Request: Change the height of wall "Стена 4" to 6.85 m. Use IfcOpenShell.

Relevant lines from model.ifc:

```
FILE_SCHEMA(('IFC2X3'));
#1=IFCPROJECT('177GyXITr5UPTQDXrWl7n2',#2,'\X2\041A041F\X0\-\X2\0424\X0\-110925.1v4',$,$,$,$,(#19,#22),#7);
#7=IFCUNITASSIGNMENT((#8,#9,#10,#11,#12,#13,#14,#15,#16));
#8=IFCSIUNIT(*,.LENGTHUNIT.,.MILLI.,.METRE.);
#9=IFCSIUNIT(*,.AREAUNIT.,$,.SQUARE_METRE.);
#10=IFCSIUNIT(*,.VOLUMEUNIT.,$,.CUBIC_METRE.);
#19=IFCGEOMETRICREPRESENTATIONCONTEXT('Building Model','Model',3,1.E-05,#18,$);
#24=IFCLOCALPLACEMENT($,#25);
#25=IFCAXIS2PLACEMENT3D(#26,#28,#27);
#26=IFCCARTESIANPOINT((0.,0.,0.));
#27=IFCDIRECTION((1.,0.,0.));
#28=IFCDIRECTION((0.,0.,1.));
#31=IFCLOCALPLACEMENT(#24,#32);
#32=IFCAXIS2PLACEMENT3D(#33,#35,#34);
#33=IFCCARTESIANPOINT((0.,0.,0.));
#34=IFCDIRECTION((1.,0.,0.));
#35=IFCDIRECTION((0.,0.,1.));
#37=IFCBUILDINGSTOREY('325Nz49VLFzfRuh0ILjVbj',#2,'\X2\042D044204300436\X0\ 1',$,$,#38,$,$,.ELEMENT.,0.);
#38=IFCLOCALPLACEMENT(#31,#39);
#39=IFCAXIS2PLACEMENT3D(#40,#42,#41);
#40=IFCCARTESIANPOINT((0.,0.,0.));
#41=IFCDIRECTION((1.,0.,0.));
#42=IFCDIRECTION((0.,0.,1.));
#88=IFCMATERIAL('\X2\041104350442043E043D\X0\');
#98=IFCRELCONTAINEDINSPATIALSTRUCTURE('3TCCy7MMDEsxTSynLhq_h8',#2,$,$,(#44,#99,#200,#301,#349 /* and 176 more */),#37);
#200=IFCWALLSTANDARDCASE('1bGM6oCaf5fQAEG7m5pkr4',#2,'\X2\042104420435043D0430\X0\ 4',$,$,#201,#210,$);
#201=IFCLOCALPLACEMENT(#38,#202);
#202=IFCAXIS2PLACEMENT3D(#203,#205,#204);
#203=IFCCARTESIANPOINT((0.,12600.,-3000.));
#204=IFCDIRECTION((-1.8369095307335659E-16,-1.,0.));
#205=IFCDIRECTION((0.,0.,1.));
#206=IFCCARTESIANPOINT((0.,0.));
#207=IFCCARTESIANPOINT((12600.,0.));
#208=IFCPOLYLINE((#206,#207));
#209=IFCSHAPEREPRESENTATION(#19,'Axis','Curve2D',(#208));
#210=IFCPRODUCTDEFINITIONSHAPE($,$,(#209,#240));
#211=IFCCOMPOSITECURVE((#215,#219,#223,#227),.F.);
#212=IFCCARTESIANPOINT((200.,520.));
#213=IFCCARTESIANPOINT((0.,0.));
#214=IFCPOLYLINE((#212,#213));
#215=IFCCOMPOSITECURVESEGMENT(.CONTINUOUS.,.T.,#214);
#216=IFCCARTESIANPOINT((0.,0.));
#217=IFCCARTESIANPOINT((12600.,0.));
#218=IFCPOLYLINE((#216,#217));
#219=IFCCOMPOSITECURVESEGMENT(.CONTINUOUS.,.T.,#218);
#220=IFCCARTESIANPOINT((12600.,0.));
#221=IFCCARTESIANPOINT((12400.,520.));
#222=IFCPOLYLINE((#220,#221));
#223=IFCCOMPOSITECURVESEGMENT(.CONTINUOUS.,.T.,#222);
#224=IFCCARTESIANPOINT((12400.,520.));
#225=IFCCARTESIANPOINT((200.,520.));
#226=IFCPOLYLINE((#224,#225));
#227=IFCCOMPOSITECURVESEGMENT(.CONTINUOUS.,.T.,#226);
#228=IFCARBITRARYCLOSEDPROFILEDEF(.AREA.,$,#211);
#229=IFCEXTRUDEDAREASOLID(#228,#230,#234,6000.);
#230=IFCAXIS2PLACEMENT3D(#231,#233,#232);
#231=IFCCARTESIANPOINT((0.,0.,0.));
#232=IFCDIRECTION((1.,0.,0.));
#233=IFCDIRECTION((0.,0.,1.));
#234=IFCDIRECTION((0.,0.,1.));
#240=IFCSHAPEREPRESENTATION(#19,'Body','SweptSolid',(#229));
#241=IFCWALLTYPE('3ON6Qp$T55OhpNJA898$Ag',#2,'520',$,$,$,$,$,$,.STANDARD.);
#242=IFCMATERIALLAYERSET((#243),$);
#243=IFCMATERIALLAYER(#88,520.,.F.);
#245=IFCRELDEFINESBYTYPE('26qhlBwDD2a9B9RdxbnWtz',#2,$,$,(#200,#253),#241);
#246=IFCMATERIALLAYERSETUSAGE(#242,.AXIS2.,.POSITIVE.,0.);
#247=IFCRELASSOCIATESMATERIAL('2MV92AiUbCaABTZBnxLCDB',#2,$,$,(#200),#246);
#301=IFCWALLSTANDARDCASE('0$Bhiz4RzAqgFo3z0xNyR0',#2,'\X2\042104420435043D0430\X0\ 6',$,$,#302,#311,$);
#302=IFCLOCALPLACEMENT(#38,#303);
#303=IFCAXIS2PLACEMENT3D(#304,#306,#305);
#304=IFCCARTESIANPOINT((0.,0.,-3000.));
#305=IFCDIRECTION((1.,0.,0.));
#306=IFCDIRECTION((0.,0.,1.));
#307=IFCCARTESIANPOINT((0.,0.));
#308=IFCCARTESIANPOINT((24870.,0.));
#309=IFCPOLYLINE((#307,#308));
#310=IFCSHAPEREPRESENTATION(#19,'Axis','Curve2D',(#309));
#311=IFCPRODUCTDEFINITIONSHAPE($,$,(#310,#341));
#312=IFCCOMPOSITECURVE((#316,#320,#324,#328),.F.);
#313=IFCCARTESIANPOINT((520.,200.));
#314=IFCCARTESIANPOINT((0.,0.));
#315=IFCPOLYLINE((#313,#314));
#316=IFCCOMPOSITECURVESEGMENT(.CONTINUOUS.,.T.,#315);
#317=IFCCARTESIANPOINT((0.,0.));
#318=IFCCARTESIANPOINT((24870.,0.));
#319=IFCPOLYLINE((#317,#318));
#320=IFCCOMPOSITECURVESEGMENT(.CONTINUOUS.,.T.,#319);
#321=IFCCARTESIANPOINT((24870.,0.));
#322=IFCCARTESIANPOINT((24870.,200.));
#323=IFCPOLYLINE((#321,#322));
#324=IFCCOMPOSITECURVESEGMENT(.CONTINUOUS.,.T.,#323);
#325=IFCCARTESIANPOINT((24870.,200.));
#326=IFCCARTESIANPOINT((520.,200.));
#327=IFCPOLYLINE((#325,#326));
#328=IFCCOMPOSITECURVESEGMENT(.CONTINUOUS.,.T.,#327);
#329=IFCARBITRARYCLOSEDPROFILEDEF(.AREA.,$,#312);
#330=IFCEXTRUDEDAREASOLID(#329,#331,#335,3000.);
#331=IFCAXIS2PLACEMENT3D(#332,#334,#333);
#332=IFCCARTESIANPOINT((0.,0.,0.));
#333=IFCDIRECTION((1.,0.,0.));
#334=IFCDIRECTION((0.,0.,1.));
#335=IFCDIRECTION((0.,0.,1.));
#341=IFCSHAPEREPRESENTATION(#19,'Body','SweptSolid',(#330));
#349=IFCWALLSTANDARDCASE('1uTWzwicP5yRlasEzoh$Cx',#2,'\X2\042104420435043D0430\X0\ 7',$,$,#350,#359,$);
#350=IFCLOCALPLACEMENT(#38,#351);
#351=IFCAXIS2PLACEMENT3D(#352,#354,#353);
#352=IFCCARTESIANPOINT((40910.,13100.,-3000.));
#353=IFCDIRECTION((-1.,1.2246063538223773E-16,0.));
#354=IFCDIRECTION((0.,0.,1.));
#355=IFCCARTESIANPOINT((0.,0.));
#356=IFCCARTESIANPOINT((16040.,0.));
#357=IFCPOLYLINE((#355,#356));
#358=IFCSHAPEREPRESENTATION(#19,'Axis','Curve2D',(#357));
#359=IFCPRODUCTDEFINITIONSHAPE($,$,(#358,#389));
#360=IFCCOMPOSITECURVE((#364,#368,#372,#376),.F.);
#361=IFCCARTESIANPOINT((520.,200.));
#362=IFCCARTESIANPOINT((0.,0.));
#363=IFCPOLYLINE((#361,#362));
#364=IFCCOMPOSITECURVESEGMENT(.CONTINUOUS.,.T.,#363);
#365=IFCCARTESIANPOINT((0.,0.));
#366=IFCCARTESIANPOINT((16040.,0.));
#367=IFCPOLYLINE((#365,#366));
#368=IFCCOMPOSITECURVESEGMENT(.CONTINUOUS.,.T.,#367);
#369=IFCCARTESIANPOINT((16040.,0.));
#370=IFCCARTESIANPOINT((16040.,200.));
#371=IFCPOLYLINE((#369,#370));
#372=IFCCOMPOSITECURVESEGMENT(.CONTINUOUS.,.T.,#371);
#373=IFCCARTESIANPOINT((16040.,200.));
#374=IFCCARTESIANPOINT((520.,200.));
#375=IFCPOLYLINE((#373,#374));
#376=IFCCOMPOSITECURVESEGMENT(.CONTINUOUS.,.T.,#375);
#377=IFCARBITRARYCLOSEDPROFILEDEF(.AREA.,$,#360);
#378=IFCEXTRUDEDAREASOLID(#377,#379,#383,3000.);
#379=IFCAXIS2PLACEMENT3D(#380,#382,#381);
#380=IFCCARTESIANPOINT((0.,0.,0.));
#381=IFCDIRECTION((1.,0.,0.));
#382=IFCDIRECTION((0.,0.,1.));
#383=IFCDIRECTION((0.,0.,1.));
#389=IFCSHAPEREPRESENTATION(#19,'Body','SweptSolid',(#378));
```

```python
import ifcopenshell
import ifcopenshell.geom
import ifcopenshell.util.shape

model = ifcopenshell.open("model.ifc")
settings = ifcopenshell.geom.settings()


def volume(element):
    """Net volume in cubic metres, openings subtracted."""
    shape = ifcopenshell.geom.create_shape(settings, element)
    return ifcopenshell.util.shape.get_volume(shape.geometry)


wall = model.by_guid("1bGM6oCaf5fQAEG7m5pkr4")
before = volume(wall)

body = next(r for r in wall.Representation.Representations if r.RepresentationIdentifier == "Body")
solid = body.Items[0]
old_height = solid.Depth
solid.Depth = 6850.0
after = volume(wall)

print(f"height {old_height:g} -> {solid.Depth:g}, volume {before:.3f} -> {after:.3f} m3")

model.write("model_edited.ifc")
```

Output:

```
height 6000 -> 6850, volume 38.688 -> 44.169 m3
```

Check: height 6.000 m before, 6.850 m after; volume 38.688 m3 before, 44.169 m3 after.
